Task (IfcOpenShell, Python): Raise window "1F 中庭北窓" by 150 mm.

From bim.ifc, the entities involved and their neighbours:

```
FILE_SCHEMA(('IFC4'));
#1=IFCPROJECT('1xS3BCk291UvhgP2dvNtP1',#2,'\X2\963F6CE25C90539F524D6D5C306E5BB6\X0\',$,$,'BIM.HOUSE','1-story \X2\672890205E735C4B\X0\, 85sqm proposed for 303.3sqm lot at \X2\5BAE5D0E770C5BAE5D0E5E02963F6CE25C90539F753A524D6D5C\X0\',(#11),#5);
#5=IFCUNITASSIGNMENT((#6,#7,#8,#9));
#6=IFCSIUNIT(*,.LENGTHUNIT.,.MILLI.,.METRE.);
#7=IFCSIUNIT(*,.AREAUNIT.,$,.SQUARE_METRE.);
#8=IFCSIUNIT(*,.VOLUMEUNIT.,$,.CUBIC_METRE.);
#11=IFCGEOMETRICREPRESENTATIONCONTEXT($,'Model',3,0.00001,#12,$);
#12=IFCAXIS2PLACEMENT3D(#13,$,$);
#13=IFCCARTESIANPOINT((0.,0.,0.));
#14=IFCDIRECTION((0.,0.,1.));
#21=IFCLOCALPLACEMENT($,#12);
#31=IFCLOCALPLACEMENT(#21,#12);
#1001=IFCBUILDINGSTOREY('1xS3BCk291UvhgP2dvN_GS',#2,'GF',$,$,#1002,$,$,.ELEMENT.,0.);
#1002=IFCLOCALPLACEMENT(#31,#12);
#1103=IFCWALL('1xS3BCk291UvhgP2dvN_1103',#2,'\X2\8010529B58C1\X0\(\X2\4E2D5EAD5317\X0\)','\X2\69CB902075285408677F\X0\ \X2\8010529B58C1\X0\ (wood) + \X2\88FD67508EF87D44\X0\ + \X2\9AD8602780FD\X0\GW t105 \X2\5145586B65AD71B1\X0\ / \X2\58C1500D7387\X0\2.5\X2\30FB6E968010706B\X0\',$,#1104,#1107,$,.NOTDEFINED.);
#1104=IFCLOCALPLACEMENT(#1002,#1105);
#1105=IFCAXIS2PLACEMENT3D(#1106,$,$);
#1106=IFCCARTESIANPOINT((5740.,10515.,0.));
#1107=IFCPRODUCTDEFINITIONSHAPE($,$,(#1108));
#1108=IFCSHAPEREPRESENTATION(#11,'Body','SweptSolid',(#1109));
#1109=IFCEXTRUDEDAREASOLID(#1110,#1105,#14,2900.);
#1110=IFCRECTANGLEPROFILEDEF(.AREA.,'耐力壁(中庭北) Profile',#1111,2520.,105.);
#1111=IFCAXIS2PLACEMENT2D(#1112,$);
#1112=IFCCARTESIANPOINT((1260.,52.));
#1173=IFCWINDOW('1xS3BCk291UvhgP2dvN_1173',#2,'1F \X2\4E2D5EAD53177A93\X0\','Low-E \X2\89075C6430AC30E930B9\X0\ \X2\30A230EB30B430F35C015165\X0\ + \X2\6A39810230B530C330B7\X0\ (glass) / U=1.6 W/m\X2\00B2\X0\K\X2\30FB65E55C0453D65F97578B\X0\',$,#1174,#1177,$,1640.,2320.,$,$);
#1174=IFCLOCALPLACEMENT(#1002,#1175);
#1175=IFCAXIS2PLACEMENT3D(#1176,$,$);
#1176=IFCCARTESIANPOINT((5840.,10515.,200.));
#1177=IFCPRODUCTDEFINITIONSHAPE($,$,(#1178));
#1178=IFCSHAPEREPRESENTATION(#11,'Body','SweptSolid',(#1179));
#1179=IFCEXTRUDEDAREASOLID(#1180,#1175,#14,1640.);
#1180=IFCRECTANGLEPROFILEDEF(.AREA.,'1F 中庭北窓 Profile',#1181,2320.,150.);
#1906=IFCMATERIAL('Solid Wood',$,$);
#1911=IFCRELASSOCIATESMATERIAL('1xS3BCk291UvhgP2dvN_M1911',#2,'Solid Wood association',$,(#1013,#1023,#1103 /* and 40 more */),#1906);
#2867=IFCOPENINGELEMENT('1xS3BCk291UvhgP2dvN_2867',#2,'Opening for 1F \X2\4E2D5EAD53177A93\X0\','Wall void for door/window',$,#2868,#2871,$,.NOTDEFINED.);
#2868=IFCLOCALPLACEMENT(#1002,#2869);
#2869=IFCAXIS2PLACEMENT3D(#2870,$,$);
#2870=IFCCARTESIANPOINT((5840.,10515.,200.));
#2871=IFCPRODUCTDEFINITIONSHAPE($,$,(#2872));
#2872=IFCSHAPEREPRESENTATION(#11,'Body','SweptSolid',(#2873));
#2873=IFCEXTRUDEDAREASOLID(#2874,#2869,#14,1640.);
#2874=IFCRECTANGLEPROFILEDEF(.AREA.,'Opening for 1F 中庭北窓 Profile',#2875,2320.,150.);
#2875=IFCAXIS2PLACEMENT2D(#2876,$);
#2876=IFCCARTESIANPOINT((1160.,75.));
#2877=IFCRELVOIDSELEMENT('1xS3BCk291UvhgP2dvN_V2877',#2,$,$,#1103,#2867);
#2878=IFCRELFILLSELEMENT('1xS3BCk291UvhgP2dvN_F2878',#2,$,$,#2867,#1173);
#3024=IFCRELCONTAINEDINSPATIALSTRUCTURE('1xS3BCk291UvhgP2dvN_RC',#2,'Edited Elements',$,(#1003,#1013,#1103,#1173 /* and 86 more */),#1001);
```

```python
import numpy as np
import ifcopenshell
import ifcopenshell.api.geometry
import ifcopenshell.util.placement
import ifcopenshell.util.unit

model = ifcopenshell.open("bim.ifc")
unit_scale = ifcopenshell.util.unit.calculate_unit_scale(model)

window = model.by_guid("1xS3BCk291UvhgP2dvN_1173")
opening = window.FillsVoids[0].RelatingOpeningElement
dz = 150.0

shift = np.array([0.0, 0.0, dz])
# The window is not placed relative to its opening, so move both.
for product in (opening, window):
    matrix = ifcopenshell.util.placement.get_local_placement(product.ObjectPlacement)
    matrix[:3, 3] += shift
    ifcopenshell.api.geometry.edit_object_placement(model, product=product, matrix=matrix, is_si=False)

print(f"moved by {dz * unit_scale:+.3f} m")

model.write("bim_updated.ifc")
```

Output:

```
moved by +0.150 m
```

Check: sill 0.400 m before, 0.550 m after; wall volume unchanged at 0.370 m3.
